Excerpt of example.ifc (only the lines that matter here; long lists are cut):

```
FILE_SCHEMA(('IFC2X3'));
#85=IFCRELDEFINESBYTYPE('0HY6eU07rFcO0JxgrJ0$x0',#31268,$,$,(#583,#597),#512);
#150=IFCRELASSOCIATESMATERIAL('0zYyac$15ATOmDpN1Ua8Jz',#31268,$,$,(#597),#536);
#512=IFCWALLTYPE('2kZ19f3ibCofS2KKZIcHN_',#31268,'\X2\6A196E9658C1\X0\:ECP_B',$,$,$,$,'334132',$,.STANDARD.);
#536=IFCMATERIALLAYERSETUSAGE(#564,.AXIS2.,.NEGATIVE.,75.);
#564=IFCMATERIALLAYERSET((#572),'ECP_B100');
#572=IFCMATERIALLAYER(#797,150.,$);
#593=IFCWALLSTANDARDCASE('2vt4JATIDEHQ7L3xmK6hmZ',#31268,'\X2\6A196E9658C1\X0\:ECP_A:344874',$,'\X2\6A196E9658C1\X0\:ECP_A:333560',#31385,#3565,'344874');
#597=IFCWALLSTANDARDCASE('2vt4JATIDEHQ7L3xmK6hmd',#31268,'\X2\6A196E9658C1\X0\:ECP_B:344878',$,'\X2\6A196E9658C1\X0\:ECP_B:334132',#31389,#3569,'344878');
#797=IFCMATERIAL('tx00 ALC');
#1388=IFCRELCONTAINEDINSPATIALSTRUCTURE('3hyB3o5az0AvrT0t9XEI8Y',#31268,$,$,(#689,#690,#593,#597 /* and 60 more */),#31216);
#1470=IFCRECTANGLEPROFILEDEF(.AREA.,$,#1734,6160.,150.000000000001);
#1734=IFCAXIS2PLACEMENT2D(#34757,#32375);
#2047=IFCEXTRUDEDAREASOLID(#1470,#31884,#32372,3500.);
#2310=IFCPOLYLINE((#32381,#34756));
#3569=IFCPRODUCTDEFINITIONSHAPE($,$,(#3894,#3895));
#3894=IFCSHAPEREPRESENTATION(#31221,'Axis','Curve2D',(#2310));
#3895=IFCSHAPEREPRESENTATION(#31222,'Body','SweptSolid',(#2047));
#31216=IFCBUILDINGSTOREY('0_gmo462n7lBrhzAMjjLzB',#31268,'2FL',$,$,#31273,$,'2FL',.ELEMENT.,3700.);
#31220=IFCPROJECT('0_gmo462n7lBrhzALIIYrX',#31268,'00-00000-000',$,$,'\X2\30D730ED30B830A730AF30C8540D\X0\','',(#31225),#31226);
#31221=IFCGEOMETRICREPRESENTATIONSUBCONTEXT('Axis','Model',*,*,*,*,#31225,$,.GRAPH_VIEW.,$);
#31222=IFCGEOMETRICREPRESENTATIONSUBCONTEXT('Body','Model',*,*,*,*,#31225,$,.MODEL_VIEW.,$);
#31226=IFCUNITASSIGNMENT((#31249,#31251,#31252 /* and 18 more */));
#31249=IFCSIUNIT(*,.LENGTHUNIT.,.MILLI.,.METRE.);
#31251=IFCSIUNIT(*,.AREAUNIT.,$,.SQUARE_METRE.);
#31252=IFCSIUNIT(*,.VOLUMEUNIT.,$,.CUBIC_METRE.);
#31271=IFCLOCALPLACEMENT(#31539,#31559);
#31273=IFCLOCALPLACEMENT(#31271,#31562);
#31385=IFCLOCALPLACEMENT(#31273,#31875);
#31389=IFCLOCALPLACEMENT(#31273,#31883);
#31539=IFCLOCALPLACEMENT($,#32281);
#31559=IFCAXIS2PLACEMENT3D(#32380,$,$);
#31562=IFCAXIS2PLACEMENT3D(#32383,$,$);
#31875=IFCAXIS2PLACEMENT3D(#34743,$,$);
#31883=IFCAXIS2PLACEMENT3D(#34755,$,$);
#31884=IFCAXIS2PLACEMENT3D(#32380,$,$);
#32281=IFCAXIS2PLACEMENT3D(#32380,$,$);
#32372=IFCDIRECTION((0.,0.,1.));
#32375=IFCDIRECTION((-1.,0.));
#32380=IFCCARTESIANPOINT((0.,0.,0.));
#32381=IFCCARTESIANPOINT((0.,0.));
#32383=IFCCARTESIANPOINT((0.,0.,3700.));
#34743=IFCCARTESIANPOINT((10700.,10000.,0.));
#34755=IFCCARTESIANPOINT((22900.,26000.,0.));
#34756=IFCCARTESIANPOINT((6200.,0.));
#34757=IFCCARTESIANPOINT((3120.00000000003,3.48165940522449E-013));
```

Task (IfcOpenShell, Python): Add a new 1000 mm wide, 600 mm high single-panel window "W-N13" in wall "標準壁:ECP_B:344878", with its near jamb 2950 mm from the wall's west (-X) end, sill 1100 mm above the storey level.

```python
import numpy as np
import ifcopenshell
import ifcopenshell.api.feature
import ifcopenshell.api.geometry
import ifcopenshell.api.root
import ifcopenshell.api.spatial
import ifcopenshell.api.type
import ifcopenshell.geom
import ifcopenshell.util.element
import ifcopenshell.util.placement
import ifcopenshell.util.representation
import ifcopenshell.util.shape
import ifcopenshell.util.unit

model = ifcopenshell.open("example.ifc")
unit_scale = ifcopenshell.util.unit.calculate_unit_scale(model)
settings = ifcopenshell.geom.settings()


def volume(element):
    """Net volume in cubic metres, openings subtracted."""
    shape = ifcopenshell.geom.create_shape(settings, element)
    return ifcopenshell.util.shape.get_volume(shape.geometry)


wall = model.by_guid("2vt4JATIDEHQ7L3xmK6hmd")
storey = ifcopenshell.util.element.get_container(wall, ifc_class="IfcBuildingStorey")
context = ifcopenshell.util.representation.get_context(model, "Model", "Body", "MODEL_VIEW")
before = volume(wall)

width, height, from_end, sill = 1, 0.6, 2.95, 1.1  # metres

# The wall runs along its own X axis, and the end named is its -X end.
wall_shape = ifcopenshell.geom.create_shape(settings, wall)
x, y, z = ifcopenshell.util.shape.get_vertices(wall_shape.geometry).T
start = x.min() + from_end
face, thickness = float(y.min()), float(y.max() - y.min())
wall_matrix = ifcopenshell.util.placement.get_local_placement(wall.ObjectPlacement)
level = ifcopenshell.util.placement.get_local_placement(storey.ObjectPlacement)[2, 3]


def in_wall(x, y):
    """Placement at x, y metres in the wall's axes, at sill height."""
    matrix = wall_matrix.copy()
    matrix[:, 3] = wall_matrix @ np.array([x / unit_scale, y / unit_scale, 0.0, 1.0])
    matrix[2, 3] = level + sill / unit_scale
    return matrix


# Opening: a box that overshoots both wall faces by 50 mm.
opening = ifcopenshell.api.root.create_entity(model, ifc_class="IfcOpeningElement")
box = ifcopenshell.api.geometry.add_wall_representation(
    model, context=context, length=width, height=height, thickness=thickness + 0.1
)
ifcopenshell.api.geometry.assign_representation(model, product=opening, representation=box)
ifcopenshell.api.geometry.edit_object_placement(model, product=opening, matrix=in_wall(start, face - 0.05), is_si=False)
ifcopenshell.api.feature.add_feature(model, feature=opening, element=wall)

window = ifcopenshell.api.root.create_entity(model, ifc_class="IfcWindow", name="W-N13")
window.OverallWidth, window.OverallHeight = width / unit_scale, height / unit_scale
body = ifcopenshell.api.geometry.add_window_representation(
    model,
    context=context,
    overall_width=window.OverallWidth,
    overall_height=window.OverallHeight,
    partition_type="SINGLE_PANEL",
)
ifcopenshell.api.geometry.assign_representation(model, product=window, representation=body)
ifcopenshell.api.spatial.assign_container(model, products=[window], relating_structure=storey)
fills = ifcopenshell.api.feature.add_filling(model, opening=opening, element=window)
fills.OwnerHistory = window.OwnerHistory  # required in IFC2X3

# IFC2X3 keeps the operation on the window style.
style = ifcopenshell.api.root.create_entity(model, ifc_class="IfcWindowStyle", name="W-N13")
style.OperationType, style.ConstructionType = "SINGLE_PANEL", "NOTDEFINED"
style.ParameterTakesPrecedence = style.Sizeable = False
ifcopenshell.api.type.assign_type(model, related_objects=[window], relating_type=style)

# Centre the window in the wall's thickness.
ifcopenshell.api.geometry.edit_object_placement(model, product=window, matrix=in_wall(start, face), is_si=False)
window_shape = ifcopenshell.geom.create_shape(settings, window)
depth = ifcopenshell.util.shape.get_vertices(window_shape.geometry)[:, 1]
offset = face + thickness / 2 - (depth.min() + depth.max()) / 2
ifcopenshell.api.geometry.edit_object_placement(model, product=window, matrix=in_wall(start, offset), is_si=False)

after = volume(wall)

print(f"wall volume {before:.3f} -> {after:.3f} m3")

model.write("example_rev.ifc")
```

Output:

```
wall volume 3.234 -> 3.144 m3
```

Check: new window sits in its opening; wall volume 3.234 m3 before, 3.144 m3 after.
